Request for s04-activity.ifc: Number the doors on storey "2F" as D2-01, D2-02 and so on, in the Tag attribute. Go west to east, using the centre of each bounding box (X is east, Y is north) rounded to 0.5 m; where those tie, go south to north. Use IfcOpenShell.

First a look at what the model holds.

```python
import ifcopenshell
import ifcopenshell.util.element
import ifcopenshell.util.placement

model = ifcopenshell.open("s04-activity.ifc")
print(model.schema)
storey = next(s for s in model.by_type("IfcBuildingStorey") if s.Name == "2F")
doors = [e for e in ifcopenshell.util.element.get_decomposition(storey) if e.is_a("IfcDoor")]
for e in sorted(doors, key=lambda e: e.id()):
    origin = ifcopenshell.util.placement.get_local_placement(e.ObjectPlacement)[:3, 3]
    print(e.id(), e.Tag, e.Name, origin.round(2) + 0.0, sep=" | ")
```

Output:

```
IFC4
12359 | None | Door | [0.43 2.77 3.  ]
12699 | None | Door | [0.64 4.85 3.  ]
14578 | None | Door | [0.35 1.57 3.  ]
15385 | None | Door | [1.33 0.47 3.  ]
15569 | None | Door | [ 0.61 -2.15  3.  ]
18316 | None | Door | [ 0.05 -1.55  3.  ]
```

```python
import ifcopenshell
import ifcopenshell.geom
import ifcopenshell.util.element
import ifcopenshell.util.shape

model = ifcopenshell.open("s04-activity.ifc")
settings = ifcopenshell.geom.settings()
settings.set("use-world-coords", True)


def centre(element):
    shape = ifcopenshell.geom.create_shape(settings, element)
    return ifcopenshell.util.shape.get_bbox_centroid(shape.geometry)


storey = next(s for s in model.by_type("IfcBuildingStorey") if s.Name == "2F")
doors = [e for e in ifcopenshell.util.element.get_decomposition(storey) if e.is_a("IfcDoor")]

# Insertion points can sit at a corner or the storey origin, so sort by the geometry (in metres).
centres = {e: centre(e) for e in doors}
doors.sort(key=lambda e: (round(centres[e][0] / 0.5), centres[e][1]))

for i, e in enumerate(doors, start=1):
    number = f"D2-{i:02d}"
    e.Tag = number
    print(e.id(), number)

model.write("s04-activity_rev.ifc")
```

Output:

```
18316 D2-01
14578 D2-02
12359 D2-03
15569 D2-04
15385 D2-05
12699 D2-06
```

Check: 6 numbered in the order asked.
